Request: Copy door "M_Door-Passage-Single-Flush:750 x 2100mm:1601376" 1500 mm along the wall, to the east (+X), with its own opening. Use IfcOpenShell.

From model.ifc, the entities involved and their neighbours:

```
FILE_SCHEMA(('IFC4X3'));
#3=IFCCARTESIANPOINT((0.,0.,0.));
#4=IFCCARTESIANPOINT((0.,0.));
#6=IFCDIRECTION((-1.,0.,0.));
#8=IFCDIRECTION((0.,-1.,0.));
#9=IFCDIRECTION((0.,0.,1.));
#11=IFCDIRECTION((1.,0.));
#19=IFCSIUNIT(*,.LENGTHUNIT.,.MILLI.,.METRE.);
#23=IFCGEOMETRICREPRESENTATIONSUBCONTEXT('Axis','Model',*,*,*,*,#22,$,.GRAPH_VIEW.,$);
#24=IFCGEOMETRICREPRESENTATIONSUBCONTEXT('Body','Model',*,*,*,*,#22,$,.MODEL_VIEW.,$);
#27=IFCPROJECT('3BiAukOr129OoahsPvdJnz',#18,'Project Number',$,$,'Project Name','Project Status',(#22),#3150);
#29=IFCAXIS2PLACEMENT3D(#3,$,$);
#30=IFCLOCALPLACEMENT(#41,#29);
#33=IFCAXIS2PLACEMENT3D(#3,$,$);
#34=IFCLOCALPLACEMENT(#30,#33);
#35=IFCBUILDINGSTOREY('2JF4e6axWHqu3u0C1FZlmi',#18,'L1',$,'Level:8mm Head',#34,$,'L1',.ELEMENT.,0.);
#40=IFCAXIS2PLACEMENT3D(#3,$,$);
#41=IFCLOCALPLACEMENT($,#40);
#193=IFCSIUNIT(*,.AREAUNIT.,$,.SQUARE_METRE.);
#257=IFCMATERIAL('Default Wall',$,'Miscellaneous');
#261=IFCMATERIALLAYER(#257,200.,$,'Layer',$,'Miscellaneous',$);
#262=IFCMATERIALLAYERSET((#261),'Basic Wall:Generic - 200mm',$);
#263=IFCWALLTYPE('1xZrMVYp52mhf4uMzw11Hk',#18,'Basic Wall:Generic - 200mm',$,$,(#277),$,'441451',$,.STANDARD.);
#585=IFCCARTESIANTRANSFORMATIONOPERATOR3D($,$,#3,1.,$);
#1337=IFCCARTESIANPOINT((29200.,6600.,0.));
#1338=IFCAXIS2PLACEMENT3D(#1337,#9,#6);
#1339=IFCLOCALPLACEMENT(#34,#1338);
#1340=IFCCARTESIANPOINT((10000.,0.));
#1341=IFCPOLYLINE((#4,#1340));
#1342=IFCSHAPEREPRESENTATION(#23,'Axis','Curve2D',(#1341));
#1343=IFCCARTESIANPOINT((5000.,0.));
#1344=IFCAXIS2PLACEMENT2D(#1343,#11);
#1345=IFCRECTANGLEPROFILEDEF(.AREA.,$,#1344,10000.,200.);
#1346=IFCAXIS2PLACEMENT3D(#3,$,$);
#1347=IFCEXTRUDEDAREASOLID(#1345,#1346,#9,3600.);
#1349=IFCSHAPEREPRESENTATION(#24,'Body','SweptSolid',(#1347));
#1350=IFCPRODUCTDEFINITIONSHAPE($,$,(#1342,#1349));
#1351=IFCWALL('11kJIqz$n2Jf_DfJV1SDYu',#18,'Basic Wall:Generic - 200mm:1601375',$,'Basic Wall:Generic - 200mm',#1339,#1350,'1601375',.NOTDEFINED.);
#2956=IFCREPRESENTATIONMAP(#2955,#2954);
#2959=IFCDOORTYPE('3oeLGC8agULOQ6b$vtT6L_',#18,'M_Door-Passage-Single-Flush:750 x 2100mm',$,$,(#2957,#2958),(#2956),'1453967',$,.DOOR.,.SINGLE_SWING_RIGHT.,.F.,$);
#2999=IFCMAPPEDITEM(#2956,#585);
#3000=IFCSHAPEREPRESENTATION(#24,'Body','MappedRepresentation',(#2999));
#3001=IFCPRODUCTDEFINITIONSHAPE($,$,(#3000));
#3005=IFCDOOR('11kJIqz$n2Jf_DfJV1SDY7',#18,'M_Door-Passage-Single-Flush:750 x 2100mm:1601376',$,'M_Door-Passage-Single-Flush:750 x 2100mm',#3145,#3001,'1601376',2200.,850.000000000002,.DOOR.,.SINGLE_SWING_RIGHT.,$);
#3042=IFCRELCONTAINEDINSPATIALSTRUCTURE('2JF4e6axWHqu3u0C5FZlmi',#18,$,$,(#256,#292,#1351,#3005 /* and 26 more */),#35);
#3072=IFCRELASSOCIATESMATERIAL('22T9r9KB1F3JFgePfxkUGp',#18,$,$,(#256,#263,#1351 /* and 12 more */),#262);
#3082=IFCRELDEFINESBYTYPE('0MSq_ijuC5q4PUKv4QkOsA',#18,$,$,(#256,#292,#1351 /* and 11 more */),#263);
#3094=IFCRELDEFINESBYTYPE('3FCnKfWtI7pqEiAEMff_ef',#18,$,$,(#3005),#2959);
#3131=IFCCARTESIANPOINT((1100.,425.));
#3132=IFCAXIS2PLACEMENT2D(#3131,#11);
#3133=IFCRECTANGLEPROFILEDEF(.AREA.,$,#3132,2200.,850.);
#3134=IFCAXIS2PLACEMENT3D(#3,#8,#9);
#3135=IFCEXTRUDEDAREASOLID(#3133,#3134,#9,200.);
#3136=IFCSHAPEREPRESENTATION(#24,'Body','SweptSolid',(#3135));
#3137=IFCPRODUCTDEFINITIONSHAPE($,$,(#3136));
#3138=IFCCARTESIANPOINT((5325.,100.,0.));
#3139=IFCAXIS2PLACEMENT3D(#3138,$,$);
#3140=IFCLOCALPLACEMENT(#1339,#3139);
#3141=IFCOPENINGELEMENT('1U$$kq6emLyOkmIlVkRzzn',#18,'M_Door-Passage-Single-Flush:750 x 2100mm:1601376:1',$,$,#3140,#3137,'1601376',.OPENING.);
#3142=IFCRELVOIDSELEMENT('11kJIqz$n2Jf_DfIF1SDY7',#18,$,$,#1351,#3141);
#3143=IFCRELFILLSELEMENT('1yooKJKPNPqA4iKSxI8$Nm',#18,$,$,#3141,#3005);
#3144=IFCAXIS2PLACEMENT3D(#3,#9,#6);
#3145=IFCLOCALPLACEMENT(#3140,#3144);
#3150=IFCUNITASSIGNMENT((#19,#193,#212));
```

```python
import ifcopenshell
import ifcopenshell.api.feature
import ifcopenshell.api.geometry
import ifcopenshell.api.root
import ifcopenshell.geom
import ifcopenshell.util.element
import ifcopenshell.util.placement
import ifcopenshell.util.shape
import ifcopenshell.util.unit

model = ifcopenshell.open("model.ifc")
unit_scale = ifcopenshell.util.unit.calculate_unit_scale(model)
settings = ifcopenshell.geom.settings()


def volume(element):
    """Net volume in cubic metres, openings subtracted."""
    shape = ifcopenshell.geom.create_shape(settings, element)
    return ifcopenshell.util.shape.get_volume(shape.geometry)


def reuse_history(source, copy):
    """copy_class also copies each property set's owner history, people and application; keep the originals."""
    for rel in copy.IsDefinedBy:
        if rel.is_a("IfcRelDefinesByProperties") and (history := rel.RelatingPropertyDefinition.OwnerHistory):
            rel.RelatingPropertyDefinition.OwnerHistory = source.OwnerHistory
            ifcopenshell.util.element.remove_deep2(model, history)


door = model.by_guid("11kJIqz$n2Jf_DfJV1SDY7")
opening = door.FillsVoids[0].RelatingOpeningElement
wall = opening.VoidsElements[0].RelatingBuildingElement
before = volume(wall)
shift = ifcopenshell.util.placement.get_local_placement(wall.ObjectPlacement)[:3, 0] * -1.5 / unit_scale

# copy_class copies the void relationship, type, container and properties, but no geometry.
new_opening = ifcopenshell.api.root.copy_class(model, product=opening)
new_opening.Representation = ifcopenshell.util.element.copy_deep(
    model, opening.Representation, exclude=["IfcGeometricRepresentationContext", "IfcRepresentationMap"]
)
new_opening.Name = "M_Door-Passage-Single-Flush:750 x 2100mm"
new_opening.Tag = None
new_door = ifcopenshell.api.root.copy_class(model, product=door)
new_door.Representation = ifcopenshell.util.element.copy_deep(
    model, door.Representation, exclude=["IfcGeometricRepresentationContext", "IfcRepresentationMap"]
)
new_door.Name = "M_Door-Passage-Single-Flush:750 x 2100mm"
new_door.Tag = None
reuse_history(door, new_door)
ifcopenshell.api.feature.add_filling(model, opening=new_opening, element=new_door)

for old, new in ((opening, new_opening), (door, new_door)):
    matrix = ifcopenshell.util.placement.get_local_placement(old.ObjectPlacement)
    matrix[:3, 3] += shift
    ifcopenshell.api.geometry.edit_object_placement(model, product=new, matrix=matrix, is_si=False)

after = volume(wall)

print(f"wall volume {before:.3f} -> {after:.3f} m3")

model.write("model_rev.ifc")
```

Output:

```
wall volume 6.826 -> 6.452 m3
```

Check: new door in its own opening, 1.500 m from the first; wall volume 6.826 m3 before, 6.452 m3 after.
